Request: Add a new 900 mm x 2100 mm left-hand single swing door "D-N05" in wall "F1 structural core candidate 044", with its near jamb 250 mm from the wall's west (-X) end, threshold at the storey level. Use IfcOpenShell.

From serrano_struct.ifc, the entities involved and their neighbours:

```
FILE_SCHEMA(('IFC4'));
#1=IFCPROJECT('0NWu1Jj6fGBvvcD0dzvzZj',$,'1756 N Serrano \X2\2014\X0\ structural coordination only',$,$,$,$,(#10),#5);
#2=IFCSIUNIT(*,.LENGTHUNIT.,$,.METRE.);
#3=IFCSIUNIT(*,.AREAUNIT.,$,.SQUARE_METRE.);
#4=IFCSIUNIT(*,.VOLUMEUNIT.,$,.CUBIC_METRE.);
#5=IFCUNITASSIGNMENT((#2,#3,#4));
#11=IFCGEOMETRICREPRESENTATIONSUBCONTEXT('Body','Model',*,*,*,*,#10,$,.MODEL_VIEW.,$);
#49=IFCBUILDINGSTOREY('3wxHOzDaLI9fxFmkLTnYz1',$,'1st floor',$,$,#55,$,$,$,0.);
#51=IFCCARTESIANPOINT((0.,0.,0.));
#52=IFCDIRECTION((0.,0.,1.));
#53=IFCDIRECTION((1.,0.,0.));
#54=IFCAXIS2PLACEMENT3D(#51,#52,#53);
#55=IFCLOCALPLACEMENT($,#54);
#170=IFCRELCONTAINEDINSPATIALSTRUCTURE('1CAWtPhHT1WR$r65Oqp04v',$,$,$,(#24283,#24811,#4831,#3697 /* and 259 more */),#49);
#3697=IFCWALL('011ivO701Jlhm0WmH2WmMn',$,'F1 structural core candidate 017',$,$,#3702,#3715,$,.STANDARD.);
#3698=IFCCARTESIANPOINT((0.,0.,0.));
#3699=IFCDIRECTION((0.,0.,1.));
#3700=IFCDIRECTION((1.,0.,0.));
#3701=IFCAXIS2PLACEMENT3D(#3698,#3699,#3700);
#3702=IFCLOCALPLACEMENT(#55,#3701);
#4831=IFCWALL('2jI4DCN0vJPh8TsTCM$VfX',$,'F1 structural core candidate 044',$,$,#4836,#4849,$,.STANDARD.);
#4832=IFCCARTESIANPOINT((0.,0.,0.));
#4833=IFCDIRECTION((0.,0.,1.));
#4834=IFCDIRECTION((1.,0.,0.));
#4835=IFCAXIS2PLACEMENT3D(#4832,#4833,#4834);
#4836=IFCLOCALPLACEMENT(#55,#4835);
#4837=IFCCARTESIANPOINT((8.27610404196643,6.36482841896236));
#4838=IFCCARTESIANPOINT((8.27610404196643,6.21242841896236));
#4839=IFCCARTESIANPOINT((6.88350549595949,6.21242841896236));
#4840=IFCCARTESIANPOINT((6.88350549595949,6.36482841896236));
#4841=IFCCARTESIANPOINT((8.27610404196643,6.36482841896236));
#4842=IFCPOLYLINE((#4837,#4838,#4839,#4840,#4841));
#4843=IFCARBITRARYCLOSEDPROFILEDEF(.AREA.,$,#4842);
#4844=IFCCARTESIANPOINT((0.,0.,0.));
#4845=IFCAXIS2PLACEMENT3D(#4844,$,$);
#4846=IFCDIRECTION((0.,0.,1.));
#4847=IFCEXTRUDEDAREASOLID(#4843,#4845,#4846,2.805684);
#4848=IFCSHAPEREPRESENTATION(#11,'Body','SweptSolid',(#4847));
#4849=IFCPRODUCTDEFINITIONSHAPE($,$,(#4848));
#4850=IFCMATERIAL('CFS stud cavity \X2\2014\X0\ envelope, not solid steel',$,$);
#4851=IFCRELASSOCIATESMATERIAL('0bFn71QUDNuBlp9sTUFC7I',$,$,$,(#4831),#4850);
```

```python
import numpy as np
import ifcopenshell
import ifcopenshell.api.feature
import ifcopenshell.api.geometry
import ifcopenshell.api.root
import ifcopenshell.api.spatial
import ifcopenshell.geom
import ifcopenshell.util.element
import ifcopenshell.util.placement
import ifcopenshell.util.representation
import ifcopenshell.util.shape
import ifcopenshell.util.unit

model = ifcopenshell.open("serrano_struct.ifc")
unit_scale = ifcopenshell.util.unit.calculate_unit_scale(model)
settings = ifcopenshell.geom.settings()


def volume(element):
    """Net volume in cubic metres, openings subtracted."""
    shape = ifcopenshell.geom.create_shape(settings, element)
    return ifcopenshell.util.shape.get_volume(shape.geometry)


wall = model.by_id(4831)
storey = ifcopenshell.util.element.get_container(wall, ifc_class="IfcBuildingStorey")
context = ifcopenshell.util.representation.get_context(model, "Model", "Body", "MODEL_VIEW")
before = volume(wall)

width, height, from_end, sill = 0.9, 2.1, 0.25, 0.0  # metres

# The wall runs along its own X axis, and the end named is its -X end.
wall_shape = ifcopenshell.geom.create_shape(settings, wall)
x, y, z = ifcopenshell.util.shape.get_vertices(wall_shape.geometry).T
start = x.min() + from_end
face, thickness = float(y.min()), float(y.max() - y.min())
wall_matrix = ifcopenshell.util.placement.get_local_placement(wall.ObjectPlacement)
level = ifcopenshell.util.placement.get_local_placement(storey.ObjectPlacement)[2, 3]


def in_wall(x, y):
    """Placement at x, y metres in the wall's axes, at sill height."""
    matrix = wall_matrix.copy()
    matrix[:, 3] = wall_matrix @ np.array([x / unit_scale, y / unit_scale, 0.0, 1.0])
    matrix[2, 3] = level + sill / unit_scale
    return matrix


# Opening: a box that overshoots both wall faces by 50 mm.
opening = ifcopenshell.api.root.create_entity(model, ifc_class="IfcOpeningElement", predefined_type="OPENING")
box = ifcopenshell.api.geometry.add_wall_representation(
    model, context=context, length=width, height=height, thickness=thickness + 0.1
)
ifcopenshell.api.geometry.assign_representation(model, product=opening, representation=box)
ifcopenshell.api.geometry.edit_object_placement(model, product=opening, matrix=in_wall(start, face - 0.05), is_si=False)
ifcopenshell.api.feature.add_feature(model, feature=opening, element=wall)

door = ifcopenshell.api.root.create_entity(model, ifc_class="IfcDoor", name="D-N05", predefined_type="DOOR")
door.OverallWidth, door.OverallHeight = width / unit_scale, height / unit_scale
door.OperationType = "SINGLE_SWING_LEFT"
body = ifcopenshell.api.geometry.add_door_representation(
    model,
    context=context,
    overall_width=door.OverallWidth,
    overall_height=door.OverallHeight,
    operation_type="SINGLE_SWING_LEFT",
    lining_properties={"LiningDepth": thickness / unit_scale, "ThresholdDepth": thickness / unit_scale},
)
ifcopenshell.api.geometry.assign_representation(model, product=door, representation=body)
ifcopenshell.api.spatial.assign_container(model, products=[door], relating_structure=storey)
ifcopenshell.api.feature.add_filling(model, opening=opening, element=door)

# The lining spans the wall, so the door starts at the wall face.
ifcopenshell.api.geometry.edit_object_placement(model, product=door, matrix=in_wall(start, face), is_si=False)

after = volume(wall)

print(f"wall volume {before:.3f} -> {after:.3f} m3")

model.write("serrano_struct-out.ifc")
```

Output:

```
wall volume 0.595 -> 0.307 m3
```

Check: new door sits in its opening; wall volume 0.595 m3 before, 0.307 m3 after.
